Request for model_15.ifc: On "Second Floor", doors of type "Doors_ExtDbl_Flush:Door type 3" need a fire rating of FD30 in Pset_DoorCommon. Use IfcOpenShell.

First a look at what the model holds.

```python
import ifcopenshell
import ifcopenshell.util.element

model = ifcopenshell.open("model_15.ifc")
print(model.schema)
storey = next(s for s in model.by_type("IfcBuildingStorey") if s.Name == "Second Floor")
doors = [e for e in ifcopenshell.util.element.get_decomposition(storey) if e.is_a("IfcDoor")]
seen = {}
for e in doors:
    element_type = ifcopenshell.util.element.get_type(e)
    key = (element_type.Name if element_type != e and element_type else None, ifcopenshell.util.element.get_pset(e, "Pset_DoorCommon", "FireRating"))
    seen[key] = seen.get(key, 0) + 1
for (name, value), count in sorted(seen.items(), key=str):
    print(count, "x", name, "|", value)
```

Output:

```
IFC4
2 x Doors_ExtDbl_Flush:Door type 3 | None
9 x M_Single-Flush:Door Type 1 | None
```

```python
import ifcopenshell
import ifcopenshell.api.pset
import ifcopenshell.util.element

model = ifcopenshell.open("model_15.ifc")

storey = next(s for s in model.by_type("IfcBuildingStorey") if s.Name == "Second Floor")
doors = [e for e in ifcopenshell.util.element.get_decomposition(storey) if e.is_a("IfcDoor")]

count = 0
for e in doors:
    element_type = ifcopenshell.util.element.get_type(e)
    if element_type in (None, e) or element_type.Name != "Doors_ExtDbl_Flush:Door type 3":
        continue
    # add_pset returns the element's existing set when there is one.
    pset = ifcopenshell.api.pset.add_pset(model, product=e, name="Pset_DoorCommon")
    ifcopenshell.api.pset.edit_pset(model, pset=pset, properties={"FireRating": "FD30"})
    count += 1

print(count, "doors updated")

model.write("model_15-out.ifc")
```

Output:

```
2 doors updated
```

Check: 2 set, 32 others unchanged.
